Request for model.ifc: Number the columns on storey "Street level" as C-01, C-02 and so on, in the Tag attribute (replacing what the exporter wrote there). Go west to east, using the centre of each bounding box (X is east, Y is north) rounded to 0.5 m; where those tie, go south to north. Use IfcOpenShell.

First a look at what the model holds.

```python
import ifcopenshell
import ifcopenshell.util.element
import ifcopenshell.util.placement

model = ifcopenshell.open("model.ifc")
print(model.schema)
storey = next(s for s in model.by_type("IfcBuildingStorey") if s.Name == "Street level")
columns = [e for e in ifcopenshell.util.element.get_decomposition(storey) if e.is_a("IfcColumn")]
for e in sorted(columns, key=lambda e: e.id()):
    origin = ifcopenshell.util.placement.get_local_placement(e.ObjectPlacement)[:3, 3]
    print(e.id(), e.Tag, e.Name, origin.round(2) + 0.0, sep=" | ")
```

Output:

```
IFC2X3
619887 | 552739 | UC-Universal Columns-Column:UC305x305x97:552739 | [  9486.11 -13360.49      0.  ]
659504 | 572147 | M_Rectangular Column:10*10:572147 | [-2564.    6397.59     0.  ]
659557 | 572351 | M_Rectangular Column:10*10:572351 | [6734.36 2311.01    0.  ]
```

```python
import ifcopenshell
import ifcopenshell.geom
import ifcopenshell.util.element
import ifcopenshell.util.shape

model = ifcopenshell.open("model.ifc")
settings = ifcopenshell.geom.settings()
settings.set("use-world-coords", True)


def centre(element):
    shape = ifcopenshell.geom.create_shape(settings, element)
    return ifcopenshell.util.shape.get_bbox_centroid(shape.geometry)


storey = next(s for s in model.by_type("IfcBuildingStorey") if s.Name == "Street level")
columns = [e for e in ifcopenshell.util.element.get_decomposition(storey) if e.is_a("IfcColumn")]

# Insertion points can sit at a corner or the storey origin, so sort by the geometry (in metres).
centres = {e: centre(e) for e in columns}
columns.sort(key=lambda e: (round(centres[e][0] / 0.5), centres[e][1]))

for i, e in enumerate(columns, start=1):
    number = f"C-{i:02d}"
    e.Tag = number
    print(e.id(), number)

model.write("model_rev.ifc")
```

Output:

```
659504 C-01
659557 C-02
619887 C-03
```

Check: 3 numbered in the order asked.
